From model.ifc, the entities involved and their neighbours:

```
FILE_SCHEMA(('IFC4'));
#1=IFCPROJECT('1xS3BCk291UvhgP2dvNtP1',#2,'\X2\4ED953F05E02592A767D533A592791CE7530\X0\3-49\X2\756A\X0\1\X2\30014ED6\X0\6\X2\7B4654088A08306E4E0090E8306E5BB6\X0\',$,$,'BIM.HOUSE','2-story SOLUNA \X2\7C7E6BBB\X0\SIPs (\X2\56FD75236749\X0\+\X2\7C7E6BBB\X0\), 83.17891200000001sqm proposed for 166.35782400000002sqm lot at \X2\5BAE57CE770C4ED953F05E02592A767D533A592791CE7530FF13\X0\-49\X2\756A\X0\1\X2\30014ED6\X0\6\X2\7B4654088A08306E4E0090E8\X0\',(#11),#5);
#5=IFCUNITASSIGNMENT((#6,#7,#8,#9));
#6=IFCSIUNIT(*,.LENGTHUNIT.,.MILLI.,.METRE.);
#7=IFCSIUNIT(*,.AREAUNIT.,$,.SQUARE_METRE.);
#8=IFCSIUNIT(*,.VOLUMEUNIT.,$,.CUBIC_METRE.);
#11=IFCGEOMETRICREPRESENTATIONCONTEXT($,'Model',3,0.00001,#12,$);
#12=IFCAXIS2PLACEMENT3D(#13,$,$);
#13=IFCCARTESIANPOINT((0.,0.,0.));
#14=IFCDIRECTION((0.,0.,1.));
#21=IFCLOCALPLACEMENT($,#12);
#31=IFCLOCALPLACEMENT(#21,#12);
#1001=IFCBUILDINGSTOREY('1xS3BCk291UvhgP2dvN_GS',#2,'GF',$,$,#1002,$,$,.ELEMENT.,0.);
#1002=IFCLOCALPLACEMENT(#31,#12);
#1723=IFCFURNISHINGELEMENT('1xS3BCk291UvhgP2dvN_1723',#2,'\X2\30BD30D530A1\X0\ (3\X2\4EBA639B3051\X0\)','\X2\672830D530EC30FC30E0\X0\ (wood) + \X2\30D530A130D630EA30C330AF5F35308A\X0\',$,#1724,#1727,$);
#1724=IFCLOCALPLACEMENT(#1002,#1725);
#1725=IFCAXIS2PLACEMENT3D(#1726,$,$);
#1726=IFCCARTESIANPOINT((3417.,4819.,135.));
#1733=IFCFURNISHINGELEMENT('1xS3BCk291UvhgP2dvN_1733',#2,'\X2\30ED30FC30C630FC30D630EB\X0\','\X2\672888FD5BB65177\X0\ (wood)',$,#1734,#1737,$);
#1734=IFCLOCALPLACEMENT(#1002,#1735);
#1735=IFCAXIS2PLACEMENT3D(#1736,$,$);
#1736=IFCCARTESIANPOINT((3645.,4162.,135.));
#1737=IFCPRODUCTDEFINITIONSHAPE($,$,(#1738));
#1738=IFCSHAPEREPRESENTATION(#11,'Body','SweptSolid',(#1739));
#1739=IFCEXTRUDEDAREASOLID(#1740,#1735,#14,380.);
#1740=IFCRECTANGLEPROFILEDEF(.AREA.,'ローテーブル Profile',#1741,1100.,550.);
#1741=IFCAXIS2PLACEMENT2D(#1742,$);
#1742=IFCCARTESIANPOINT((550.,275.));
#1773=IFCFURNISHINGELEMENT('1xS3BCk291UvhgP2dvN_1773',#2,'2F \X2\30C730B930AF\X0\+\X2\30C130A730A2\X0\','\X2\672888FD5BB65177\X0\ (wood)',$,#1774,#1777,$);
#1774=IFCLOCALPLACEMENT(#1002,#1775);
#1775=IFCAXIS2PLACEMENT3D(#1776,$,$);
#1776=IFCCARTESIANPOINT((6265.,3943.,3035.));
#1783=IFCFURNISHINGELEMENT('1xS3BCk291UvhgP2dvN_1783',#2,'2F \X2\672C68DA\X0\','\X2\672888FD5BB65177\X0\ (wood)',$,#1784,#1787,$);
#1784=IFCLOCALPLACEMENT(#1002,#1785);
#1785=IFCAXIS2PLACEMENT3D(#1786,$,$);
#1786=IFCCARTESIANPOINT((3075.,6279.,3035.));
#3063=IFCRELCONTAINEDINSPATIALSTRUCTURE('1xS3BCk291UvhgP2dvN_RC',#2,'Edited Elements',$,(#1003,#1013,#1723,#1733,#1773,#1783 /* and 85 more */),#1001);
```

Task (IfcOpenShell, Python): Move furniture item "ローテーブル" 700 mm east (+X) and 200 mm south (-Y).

```python
import ifcopenshell
import ifcopenshell.api.geometry
import ifcopenshell.util.placement
import ifcopenshell.util.unit

model = ifcopenshell.open("model.ifc")
unit_scale = ifcopenshell.util.unit.calculate_unit_scale(model)

item = model.by_id(1733)
matrix = ifcopenshell.util.placement.get_local_placement(item.ObjectPlacement)
matrix[0, 3] += 0.7 / unit_scale
matrix[1, 3] -= 0.2 / unit_scale
ifcopenshell.api.geometry.edit_object_placement(model, product=item, matrix=matrix, is_si=False)

print(ifcopenshell.util.placement.get_local_placement(item.ObjectPlacement).round(3) + 0.0)

model.write("model-out.ifc")
```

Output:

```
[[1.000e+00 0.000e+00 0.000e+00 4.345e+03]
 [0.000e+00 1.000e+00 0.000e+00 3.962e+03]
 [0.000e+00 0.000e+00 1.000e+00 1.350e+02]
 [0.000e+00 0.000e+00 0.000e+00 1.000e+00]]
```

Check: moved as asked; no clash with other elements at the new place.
